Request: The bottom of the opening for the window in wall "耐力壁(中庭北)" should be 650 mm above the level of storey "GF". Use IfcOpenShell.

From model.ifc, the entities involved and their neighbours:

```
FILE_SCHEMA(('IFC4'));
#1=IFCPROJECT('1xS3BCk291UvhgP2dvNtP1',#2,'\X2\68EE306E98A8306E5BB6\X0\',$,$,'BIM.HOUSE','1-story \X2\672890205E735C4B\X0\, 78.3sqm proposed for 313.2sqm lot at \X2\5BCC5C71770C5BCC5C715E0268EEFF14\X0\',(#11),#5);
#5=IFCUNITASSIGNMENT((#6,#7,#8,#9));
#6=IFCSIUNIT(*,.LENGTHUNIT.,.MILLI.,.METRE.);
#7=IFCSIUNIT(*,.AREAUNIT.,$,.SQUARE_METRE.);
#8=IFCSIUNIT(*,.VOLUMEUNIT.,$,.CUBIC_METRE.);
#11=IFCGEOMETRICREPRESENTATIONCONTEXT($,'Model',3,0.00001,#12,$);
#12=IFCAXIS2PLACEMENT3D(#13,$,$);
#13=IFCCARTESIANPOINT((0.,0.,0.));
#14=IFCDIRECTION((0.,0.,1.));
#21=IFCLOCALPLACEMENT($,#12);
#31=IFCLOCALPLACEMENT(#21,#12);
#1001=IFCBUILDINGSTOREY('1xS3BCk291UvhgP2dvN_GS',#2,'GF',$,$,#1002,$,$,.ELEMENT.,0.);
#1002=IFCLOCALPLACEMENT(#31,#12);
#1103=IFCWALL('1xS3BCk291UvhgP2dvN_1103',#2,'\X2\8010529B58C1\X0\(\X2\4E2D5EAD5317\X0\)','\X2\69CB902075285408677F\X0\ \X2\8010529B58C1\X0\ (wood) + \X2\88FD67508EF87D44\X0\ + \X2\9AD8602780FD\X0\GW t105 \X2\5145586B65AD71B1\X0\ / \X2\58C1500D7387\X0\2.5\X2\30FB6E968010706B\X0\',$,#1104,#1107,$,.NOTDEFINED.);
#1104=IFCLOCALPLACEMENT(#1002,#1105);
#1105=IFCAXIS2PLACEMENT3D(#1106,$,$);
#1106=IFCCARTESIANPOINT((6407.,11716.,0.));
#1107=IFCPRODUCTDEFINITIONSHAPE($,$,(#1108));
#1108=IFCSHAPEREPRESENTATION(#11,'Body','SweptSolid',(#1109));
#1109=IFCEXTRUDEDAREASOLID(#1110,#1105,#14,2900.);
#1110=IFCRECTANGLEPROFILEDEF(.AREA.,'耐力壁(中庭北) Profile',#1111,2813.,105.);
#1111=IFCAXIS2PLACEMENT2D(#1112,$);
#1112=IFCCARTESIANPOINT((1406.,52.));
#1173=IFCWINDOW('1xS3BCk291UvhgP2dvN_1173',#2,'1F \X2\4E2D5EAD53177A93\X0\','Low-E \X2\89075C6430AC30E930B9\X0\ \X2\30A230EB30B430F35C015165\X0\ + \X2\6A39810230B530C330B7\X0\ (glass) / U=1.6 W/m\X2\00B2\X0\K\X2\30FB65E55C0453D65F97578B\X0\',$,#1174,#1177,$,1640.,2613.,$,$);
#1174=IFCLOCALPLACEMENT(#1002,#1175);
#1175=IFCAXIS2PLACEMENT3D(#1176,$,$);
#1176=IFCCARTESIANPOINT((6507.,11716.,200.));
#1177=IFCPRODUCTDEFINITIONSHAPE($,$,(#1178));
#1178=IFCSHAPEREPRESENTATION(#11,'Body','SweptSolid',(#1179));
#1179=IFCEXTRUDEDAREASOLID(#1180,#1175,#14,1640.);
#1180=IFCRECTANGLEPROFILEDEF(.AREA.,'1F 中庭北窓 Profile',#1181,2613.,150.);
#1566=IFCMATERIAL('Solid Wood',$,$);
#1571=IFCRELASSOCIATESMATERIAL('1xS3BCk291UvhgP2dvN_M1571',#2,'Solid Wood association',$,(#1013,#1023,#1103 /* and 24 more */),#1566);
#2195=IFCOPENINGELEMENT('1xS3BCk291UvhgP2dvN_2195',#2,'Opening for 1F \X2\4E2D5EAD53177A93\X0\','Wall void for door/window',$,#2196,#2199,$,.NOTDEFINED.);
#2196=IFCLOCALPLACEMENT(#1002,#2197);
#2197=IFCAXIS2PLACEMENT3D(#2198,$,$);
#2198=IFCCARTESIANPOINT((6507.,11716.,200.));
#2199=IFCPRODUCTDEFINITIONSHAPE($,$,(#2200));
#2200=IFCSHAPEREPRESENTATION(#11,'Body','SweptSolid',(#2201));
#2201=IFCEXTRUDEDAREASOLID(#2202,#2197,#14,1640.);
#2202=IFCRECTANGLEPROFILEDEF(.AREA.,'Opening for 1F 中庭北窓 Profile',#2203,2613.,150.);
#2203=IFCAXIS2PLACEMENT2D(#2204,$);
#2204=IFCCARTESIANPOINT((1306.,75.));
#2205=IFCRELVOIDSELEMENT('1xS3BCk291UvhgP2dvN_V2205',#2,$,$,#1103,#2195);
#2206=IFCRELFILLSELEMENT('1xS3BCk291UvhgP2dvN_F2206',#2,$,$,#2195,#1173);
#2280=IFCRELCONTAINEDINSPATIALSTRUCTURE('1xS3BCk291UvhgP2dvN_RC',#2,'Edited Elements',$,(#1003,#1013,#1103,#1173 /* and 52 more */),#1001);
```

```python
import numpy as np
import ifcopenshell
import ifcopenshell.api.geometry
import ifcopenshell.geom
import ifcopenshell.util.element
import ifcopenshell.util.placement
import ifcopenshell.util.shape
import ifcopenshell.util.unit

model = ifcopenshell.open("model.ifc")
unit_scale = ifcopenshell.util.unit.calculate_unit_scale(model)

window = model.by_id(1173)
opening = window.FillsVoids[0].RelatingOpeningElement
storey = ifcopenshell.util.element.get_container(window, ifc_class="IfcBuildingStorey")
level = ifcopenshell.util.placement.get_local_placement(storey.ObjectPlacement)[2, 3]

# The opening's origin need not be at the sill, so measure its lowest point.
shape = ifcopenshell.geom.create_shape(ifcopenshell.geom.settings(), opening)
bottom = ifcopenshell.util.shape.get_shape_bottom_elevation(shape, shape.geometry) / unit_scale
dz = level + 650.0 - bottom

shift = np.array([0.0, 0.0, dz])
# The window is not placed relative to its opening, so move both.
for product in (opening, window):
    matrix = ifcopenshell.util.placement.get_local_placement(product.ObjectPlacement)
    matrix[:3, 3] += shift
    ifcopenshell.api.geometry.edit_object_placement(model, product=product, matrix=matrix, is_si=False)

print(f"moved by {dz * unit_scale:+.3f} m")

model.write("model_updated.ifc")
```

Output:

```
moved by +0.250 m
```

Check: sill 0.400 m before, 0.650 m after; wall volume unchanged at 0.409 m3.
